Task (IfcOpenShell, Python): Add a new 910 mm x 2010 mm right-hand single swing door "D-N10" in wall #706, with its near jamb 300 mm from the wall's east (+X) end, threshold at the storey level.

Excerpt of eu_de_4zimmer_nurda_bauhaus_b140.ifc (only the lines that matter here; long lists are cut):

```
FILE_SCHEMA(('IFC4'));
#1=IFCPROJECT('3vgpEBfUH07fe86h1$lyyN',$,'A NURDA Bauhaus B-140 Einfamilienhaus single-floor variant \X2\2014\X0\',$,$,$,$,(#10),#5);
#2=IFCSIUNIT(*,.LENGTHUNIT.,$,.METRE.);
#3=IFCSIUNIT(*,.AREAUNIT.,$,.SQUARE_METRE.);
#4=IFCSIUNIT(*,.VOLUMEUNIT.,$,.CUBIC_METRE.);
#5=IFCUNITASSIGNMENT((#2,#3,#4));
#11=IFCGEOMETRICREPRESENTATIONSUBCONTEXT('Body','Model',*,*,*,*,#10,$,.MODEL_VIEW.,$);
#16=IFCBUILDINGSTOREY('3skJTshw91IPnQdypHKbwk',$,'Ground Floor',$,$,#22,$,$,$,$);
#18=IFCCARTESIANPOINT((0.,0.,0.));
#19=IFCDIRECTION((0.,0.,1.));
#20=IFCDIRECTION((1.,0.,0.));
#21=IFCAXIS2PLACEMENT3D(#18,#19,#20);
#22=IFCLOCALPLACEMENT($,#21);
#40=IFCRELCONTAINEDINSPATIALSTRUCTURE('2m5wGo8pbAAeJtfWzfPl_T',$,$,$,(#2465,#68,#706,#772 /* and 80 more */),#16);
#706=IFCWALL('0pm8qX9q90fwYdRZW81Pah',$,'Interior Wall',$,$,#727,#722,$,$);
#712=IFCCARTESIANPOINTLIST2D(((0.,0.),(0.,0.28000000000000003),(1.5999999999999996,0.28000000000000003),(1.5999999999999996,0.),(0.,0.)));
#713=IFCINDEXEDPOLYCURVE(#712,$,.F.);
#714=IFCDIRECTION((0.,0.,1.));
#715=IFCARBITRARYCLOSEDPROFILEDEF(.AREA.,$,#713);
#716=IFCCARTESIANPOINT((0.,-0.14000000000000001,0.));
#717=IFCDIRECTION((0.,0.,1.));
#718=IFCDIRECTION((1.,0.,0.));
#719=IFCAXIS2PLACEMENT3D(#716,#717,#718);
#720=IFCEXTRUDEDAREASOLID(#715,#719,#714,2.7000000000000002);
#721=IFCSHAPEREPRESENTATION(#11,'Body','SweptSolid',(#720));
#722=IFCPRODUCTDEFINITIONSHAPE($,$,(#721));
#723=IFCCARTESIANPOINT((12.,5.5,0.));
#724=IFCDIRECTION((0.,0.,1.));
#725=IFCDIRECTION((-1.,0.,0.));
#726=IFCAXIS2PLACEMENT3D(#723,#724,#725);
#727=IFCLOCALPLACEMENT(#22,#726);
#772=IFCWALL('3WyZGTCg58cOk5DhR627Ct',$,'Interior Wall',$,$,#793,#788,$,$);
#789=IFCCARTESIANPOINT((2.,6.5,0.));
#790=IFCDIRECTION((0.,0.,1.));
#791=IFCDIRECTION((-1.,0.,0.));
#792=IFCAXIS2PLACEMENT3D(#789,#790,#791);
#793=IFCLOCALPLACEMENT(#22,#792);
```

```python
import numpy as np
import ifcopenshell
import ifcopenshell.api.feature
import ifcopenshell.api.geometry
import ifcopenshell.api.root
import ifcopenshell.api.spatial
import ifcopenshell.geom
import ifcopenshell.util.element
import ifcopenshell.util.placement
import ifcopenshell.util.representation
import ifcopenshell.util.shape
import ifcopenshell.util.unit

model = ifcopenshell.open("eu_de_4zimmer_nurda_bauhaus_b140.ifc")
unit_scale = ifcopenshell.util.unit.calculate_unit_scale(model)
settings = ifcopenshell.geom.settings()


def volume(element):
    """Net volume in cubic metres, openings subtracted."""
    shape = ifcopenshell.geom.create_shape(settings, element)
    return ifcopenshell.util.shape.get_volume(shape.geometry)


wall = model.by_guid("0pm8qX9q90fwYdRZW81Pah")
storey = ifcopenshell.util.element.get_container(wall, ifc_class="IfcBuildingStorey")
context = ifcopenshell.util.representation.get_context(model, "Model", "Body", "MODEL_VIEW")
before = volume(wall)

width, height, from_end, sill = 0.91, 2.01, 0.3, 0.0  # metres

# The wall runs along its own X axis, and the end named is its -X end.
wall_shape = ifcopenshell.geom.create_shape(settings, wall)
x, y, z = ifcopenshell.util.shape.get_vertices(wall_shape.geometry).T
start = x.min() + from_end
face, thickness = float(y.min()), float(y.max() - y.min())
wall_matrix = ifcopenshell.util.placement.get_local_placement(wall.ObjectPlacement)
level = ifcopenshell.util.placement.get_local_placement(storey.ObjectPlacement)[2, 3]


def in_wall(x, y):
    """Placement at x, y metres in the wall's axes, at sill height."""
    matrix = wall_matrix.copy()
    matrix[:, 3] = wall_matrix @ np.array([x / unit_scale, y / unit_scale, 0.0, 1.0])
    matrix[2, 3] = level + sill / unit_scale
    return matrix


# Opening: a box that overshoots both wall faces by 50 mm.
opening = ifcopenshell.api.root.create_entity(model, ifc_class="IfcOpeningElement", predefined_type="OPENING")
box = ifcopenshell.api.geometry.add_wall_representation(
    model, context=context, length=width, height=height, thickness=thickness + 0.1
)
ifcopenshell.api.geometry.assign_representation(model, product=opening, representation=box)
ifcopenshell.api.geometry.edit_object_placement(model, product=opening, matrix=in_wall(start, face - 0.05), is_si=False)
ifcopenshell.api.feature.add_feature(model, feature=opening, element=wall)

door = ifcopenshell.api.root.create_entity(model, ifc_class="IfcDoor", name="D-N10", predefined_type="DOOR")
door.OverallWidth, door.OverallHeight = width / unit_scale, height / unit_scale
door.OperationType = "SINGLE_SWING_RIGHT"
body = ifcopenshell.api.geometry.add_door_representation(
    model,
    context=context,
    overall_width=door.OverallWidth,
    overall_height=door.OverallHeight,
    operation_type="SINGLE_SWING_RIGHT",
    lining_properties={"LiningDepth": thickness / unit_scale, "ThresholdDepth": thickness / unit_scale},
)
ifcopenshell.api.geometry.assign_representation(model, product=door, representation=body)
ifcopenshell.api.spatial.assign_container(model, products=[door], relating_structure=storey)
ifcopenshell.api.feature.add_filling(model, opening=opening, element=door)

# The lining spans the wall, so the door starts at the wall face.
ifcopenshell.api.geometry.edit_object_placement(model, product=door, matrix=in_wall(start, face), is_si=False)

after = volume(wall)

print(f"wall volume {before:.3f} -> {after:.3f} m3")

model.write("eu_de_4zimmer_nurda_bauhaus_b140_updated.ifc")
```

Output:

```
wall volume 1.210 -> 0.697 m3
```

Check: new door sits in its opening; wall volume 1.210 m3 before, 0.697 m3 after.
